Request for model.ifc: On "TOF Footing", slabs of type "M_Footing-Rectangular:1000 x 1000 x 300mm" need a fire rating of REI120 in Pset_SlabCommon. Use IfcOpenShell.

First a look at what the model holds.

```python
import ifcopenshell
import ifcopenshell.util.element

model = ifcopenshell.open("model.ifc")
print(model.schema)
storey = next(s for s in model.by_type("IfcBuildingStorey") if s.Name == "TOF Footing")
slabs = [e for e in ifcopenshell.util.element.get_decomposition(storey) if e.is_a("IfcSlab")]
seen = {}
for e in slabs:
    element_type = ifcopenshell.util.element.get_type(e)
    key = (element_type.Name if element_type != e and element_type else None, ifcopenshell.util.element.get_pset(e, "Pset_SlabCommon", "FireRating"))
    seen[key] = seen.get(key, 0) + 1
for (name, value), count in sorted(seen.items(), key=str):
    print(count, "x", name, "|", value)
```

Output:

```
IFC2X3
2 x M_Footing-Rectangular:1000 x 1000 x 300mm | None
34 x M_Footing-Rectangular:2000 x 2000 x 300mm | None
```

```python
import ifcopenshell
import ifcopenshell.api.pset
import ifcopenshell.util.element

model = ifcopenshell.open("model.ifc")

storey = next(s for s in model.by_type("IfcBuildingStorey") if s.Name == "TOF Footing")
slabs = [e for e in ifcopenshell.util.element.get_decomposition(storey) if e.is_a("IfcSlab")]

count = 0
for e in slabs:
    element_type = ifcopenshell.util.element.get_type(e)
    if element_type in (None, e) or element_type.Name != "M_Footing-Rectangular:1000 x 1000 x 300mm":
        continue
    # add_pset returns the element's existing set when there is one.
    pset = ifcopenshell.api.pset.add_pset(model, product=e, name="Pset_SlabCommon")
    ifcopenshell.api.pset.edit_pset(model, pset=pset, properties={"FireRating": "REI120"})
    count += 1

print(count, "slabs updated")

model.write("model_v2.ifc")
```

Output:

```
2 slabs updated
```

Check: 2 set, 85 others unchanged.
